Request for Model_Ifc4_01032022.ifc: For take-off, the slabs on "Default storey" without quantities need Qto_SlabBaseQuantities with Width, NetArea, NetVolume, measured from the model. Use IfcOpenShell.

First a look at what the model holds.

```python
import ifcopenshell
import ifcopenshell.util.element
import ifcopenshell.util.unit

model = ifcopenshell.open("Model_Ifc4_01032022.ifc")
print(model.schema)
for unit_type in ("LENGTHUNIT", "AREAUNIT", "VOLUMEUNIT"):
    print(unit_type, ifcopenshell.util.unit.calculate_unit_scale(model, unit_type))
storey = next(s for s in model.by_type("IfcBuildingStorey") if s.Name == "Default storey")
slabs = [e for e in ifcopenshell.util.element.get_decomposition(storey) if e.is_a("IfcSlab")]
for e in sorted(slabs, key=lambda e: e.id()):
    print(e.id(), e.is_a(), e.Name, list(ifcopenshell.util.element.get_psets(e, qtos_only=True)), sep=" | ")
```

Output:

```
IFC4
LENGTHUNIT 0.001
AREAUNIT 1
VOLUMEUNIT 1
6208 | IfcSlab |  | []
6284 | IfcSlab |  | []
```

```python
import ifcopenshell
import ifcopenshell.api.pset
import ifcopenshell.geom
import ifcopenshell.util.element
import ifcopenshell.util.shape
import ifcopenshell.util.unit

model = ifcopenshell.open("Model_Ifc4_01032022.ifc")
unit_scale = ifcopenshell.util.unit.calculate_unit_scale(model)
area_scale = ifcopenshell.util.unit.calculate_unit_scale(model, "AREAUNIT")
volume_scale = ifcopenshell.util.unit.calculate_unit_scale(model, "VOLUMEUNIT")
settings = ifcopenshell.geom.settings()

storey = next(s for s in model.by_type("IfcBuildingStorey") if s.Name == "Default storey")
slabs = [e for e in ifcopenshell.util.element.get_decomposition(storey) if e.is_a("IfcSlab")]

for e in sorted(slabs, key=lambda e: e.id()):
    if ifcopenshell.util.element.get_psets(e, qtos_only=True, should_inherit=False):
        continue
    # Geometry comes back in metres, in the element's own axes.
    shape = ifcopenshell.geom.create_shape(settings, e)
    values = {
        "Width": ifcopenshell.util.shape.get_z(shape.geometry) / unit_scale,
        "NetArea": ifcopenshell.util.shape.get_footprint_area(shape.geometry) / area_scale,
        "NetVolume": ifcopenshell.util.shape.get_volume(shape.geometry) / volume_scale,
    }
    qto = ifcopenshell.api.pset.add_qto(model, product=e, name="Qto_SlabBaseQuantities")
    ifcopenshell.api.pset.edit_qto(model, qto=qto, properties=values)
    print(e.id(), {k: round(v, 3) for k, v in values.items()})

model.write("Model_Ifc4_01032022_rev.ifc")
```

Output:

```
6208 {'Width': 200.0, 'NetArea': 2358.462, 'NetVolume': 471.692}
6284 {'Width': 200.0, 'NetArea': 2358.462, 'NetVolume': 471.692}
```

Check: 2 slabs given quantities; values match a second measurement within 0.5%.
